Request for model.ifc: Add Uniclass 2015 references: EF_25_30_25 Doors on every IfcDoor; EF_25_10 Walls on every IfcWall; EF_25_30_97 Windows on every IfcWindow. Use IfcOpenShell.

First a look at what the model holds.

```python
import ifcopenshell

model = ifcopenshell.open("model.ifc")
print(model.schema)
print("classifications:", [c.Name for c in model.by_type("IfcClassification")])
for ifc_class in ("IfcDoor", "IfcRoof", "IfcStair", "IfcWall", "IfcWindow"):
    print(ifc_class, len(model.by_type(ifc_class)))
```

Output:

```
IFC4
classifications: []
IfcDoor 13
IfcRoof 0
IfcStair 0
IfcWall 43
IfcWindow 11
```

```python
import ifcopenshell
import ifcopenshell.api.classification

model = ifcopenshell.open("model.ifc")

system = ifcopenshell.api.classification.add_classification(model, classification="Uniclass 2015")

codes = {
    "IfcDoor": ("EF_25_30_25", "Doors"),
    "IfcWall": ("EF_25_10", "Walls"),
    "IfcWindow": ("EF_25_30_97", "Windows"),
}
for ifc_class, (code, name) in codes.items():
    products = model.by_type(ifc_class)
    ifcopenshell.api.classification.add_reference(
        model, products=products, classification=system, identification=code, name=name
    )
    print(code, len(products))

model.write("model_rev.ifc")
```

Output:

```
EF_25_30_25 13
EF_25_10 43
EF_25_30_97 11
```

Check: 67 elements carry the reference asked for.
